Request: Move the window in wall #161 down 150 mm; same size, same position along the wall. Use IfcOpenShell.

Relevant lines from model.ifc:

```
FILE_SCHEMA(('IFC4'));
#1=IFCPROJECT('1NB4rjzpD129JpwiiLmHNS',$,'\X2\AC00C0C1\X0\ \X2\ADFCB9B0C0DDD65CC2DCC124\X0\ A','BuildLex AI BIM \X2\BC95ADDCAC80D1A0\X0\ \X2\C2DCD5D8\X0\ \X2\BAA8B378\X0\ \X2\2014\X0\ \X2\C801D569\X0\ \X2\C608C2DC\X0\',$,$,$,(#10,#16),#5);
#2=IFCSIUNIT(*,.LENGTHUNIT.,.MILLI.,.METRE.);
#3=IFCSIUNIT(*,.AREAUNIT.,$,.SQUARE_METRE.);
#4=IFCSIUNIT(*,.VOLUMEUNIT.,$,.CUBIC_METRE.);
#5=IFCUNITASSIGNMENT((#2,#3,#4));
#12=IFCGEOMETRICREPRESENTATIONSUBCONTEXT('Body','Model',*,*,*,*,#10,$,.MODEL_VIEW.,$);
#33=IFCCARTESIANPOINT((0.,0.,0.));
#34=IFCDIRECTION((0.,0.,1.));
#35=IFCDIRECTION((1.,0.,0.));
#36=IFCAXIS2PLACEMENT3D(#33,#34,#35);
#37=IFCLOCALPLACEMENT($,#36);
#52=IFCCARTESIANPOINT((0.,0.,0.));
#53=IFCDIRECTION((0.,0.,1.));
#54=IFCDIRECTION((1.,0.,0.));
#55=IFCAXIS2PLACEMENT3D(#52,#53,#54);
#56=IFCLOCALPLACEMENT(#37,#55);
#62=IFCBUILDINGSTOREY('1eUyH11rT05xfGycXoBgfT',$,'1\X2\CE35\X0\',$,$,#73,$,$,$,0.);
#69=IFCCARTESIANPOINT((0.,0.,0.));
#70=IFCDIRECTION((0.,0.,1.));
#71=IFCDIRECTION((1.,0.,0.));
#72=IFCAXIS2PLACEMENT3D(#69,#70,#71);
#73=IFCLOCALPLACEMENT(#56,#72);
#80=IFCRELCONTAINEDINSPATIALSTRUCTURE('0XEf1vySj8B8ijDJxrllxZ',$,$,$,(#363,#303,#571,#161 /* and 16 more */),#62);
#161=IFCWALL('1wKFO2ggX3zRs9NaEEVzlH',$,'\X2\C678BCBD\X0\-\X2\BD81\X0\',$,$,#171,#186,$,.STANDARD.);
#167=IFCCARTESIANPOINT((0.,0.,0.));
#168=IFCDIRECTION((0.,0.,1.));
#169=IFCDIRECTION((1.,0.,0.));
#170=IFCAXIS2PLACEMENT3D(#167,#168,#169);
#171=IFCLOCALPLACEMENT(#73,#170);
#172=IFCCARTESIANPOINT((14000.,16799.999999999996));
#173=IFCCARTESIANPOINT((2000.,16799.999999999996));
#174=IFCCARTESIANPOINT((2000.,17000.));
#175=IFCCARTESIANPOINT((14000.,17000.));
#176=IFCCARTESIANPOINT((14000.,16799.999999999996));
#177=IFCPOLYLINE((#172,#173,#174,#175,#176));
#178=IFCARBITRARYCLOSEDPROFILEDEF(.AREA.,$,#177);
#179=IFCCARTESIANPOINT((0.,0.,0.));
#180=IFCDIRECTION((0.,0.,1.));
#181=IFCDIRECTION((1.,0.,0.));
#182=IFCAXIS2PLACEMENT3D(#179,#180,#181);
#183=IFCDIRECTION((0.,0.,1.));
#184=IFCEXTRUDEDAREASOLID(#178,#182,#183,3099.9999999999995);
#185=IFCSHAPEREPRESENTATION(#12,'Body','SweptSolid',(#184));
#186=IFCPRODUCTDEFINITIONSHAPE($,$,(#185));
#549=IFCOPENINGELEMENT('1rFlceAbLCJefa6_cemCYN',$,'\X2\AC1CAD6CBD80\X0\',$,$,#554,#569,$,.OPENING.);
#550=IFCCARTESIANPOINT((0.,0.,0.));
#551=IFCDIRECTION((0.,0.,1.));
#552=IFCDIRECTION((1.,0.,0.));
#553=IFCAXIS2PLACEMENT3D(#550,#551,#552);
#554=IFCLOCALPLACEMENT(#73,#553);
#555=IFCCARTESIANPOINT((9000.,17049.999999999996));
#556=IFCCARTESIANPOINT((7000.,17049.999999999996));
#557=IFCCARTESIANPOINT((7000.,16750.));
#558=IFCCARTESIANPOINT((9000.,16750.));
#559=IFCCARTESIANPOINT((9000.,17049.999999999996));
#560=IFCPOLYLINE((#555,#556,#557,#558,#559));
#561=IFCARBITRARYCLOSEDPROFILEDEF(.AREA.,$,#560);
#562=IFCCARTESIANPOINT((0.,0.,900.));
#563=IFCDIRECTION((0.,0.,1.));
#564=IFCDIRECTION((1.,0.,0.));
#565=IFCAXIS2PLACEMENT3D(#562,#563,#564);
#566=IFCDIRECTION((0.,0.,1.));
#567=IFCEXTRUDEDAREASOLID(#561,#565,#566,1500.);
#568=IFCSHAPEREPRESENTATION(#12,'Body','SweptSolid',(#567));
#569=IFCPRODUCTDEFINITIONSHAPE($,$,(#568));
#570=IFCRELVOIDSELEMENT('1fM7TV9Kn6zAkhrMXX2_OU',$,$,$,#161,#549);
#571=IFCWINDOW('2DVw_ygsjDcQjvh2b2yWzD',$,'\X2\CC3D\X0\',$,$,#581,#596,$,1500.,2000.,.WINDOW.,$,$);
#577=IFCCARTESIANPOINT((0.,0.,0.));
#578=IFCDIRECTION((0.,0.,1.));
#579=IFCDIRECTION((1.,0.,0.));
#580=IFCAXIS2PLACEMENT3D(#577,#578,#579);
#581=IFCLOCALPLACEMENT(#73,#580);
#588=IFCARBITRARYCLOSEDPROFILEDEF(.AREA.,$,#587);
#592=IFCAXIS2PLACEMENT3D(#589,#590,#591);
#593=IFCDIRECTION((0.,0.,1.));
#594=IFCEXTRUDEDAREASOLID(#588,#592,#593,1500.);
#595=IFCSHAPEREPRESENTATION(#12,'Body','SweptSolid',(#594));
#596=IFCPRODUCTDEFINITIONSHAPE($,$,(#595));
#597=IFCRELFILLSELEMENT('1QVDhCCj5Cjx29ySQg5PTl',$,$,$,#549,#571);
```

```python
import numpy as np
import ifcopenshell
import ifcopenshell.api.geometry
import ifcopenshell.util.placement
import ifcopenshell.util.unit

model = ifcopenshell.open("model.ifc")
unit_scale = ifcopenshell.util.unit.calculate_unit_scale(model)

window = model.by_id(571)
opening = window.FillsVoids[0].RelatingOpeningElement
dz = -0.15 / unit_scale

shift = np.array([0.0, 0.0, dz])
# The window is not placed relative to its opening, so move both.
for product in (opening, window):
    matrix = ifcopenshell.util.placement.get_local_placement(product.ObjectPlacement)
    matrix[:3, 3] += shift
    ifcopenshell.api.geometry.edit_object_placement(model, product=product, matrix=matrix, is_si=False)

print(f"moved by {dz * unit_scale:+.3f} m")

model.write("model_updated.ifc")
```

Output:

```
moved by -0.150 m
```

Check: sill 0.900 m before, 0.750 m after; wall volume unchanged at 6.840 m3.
